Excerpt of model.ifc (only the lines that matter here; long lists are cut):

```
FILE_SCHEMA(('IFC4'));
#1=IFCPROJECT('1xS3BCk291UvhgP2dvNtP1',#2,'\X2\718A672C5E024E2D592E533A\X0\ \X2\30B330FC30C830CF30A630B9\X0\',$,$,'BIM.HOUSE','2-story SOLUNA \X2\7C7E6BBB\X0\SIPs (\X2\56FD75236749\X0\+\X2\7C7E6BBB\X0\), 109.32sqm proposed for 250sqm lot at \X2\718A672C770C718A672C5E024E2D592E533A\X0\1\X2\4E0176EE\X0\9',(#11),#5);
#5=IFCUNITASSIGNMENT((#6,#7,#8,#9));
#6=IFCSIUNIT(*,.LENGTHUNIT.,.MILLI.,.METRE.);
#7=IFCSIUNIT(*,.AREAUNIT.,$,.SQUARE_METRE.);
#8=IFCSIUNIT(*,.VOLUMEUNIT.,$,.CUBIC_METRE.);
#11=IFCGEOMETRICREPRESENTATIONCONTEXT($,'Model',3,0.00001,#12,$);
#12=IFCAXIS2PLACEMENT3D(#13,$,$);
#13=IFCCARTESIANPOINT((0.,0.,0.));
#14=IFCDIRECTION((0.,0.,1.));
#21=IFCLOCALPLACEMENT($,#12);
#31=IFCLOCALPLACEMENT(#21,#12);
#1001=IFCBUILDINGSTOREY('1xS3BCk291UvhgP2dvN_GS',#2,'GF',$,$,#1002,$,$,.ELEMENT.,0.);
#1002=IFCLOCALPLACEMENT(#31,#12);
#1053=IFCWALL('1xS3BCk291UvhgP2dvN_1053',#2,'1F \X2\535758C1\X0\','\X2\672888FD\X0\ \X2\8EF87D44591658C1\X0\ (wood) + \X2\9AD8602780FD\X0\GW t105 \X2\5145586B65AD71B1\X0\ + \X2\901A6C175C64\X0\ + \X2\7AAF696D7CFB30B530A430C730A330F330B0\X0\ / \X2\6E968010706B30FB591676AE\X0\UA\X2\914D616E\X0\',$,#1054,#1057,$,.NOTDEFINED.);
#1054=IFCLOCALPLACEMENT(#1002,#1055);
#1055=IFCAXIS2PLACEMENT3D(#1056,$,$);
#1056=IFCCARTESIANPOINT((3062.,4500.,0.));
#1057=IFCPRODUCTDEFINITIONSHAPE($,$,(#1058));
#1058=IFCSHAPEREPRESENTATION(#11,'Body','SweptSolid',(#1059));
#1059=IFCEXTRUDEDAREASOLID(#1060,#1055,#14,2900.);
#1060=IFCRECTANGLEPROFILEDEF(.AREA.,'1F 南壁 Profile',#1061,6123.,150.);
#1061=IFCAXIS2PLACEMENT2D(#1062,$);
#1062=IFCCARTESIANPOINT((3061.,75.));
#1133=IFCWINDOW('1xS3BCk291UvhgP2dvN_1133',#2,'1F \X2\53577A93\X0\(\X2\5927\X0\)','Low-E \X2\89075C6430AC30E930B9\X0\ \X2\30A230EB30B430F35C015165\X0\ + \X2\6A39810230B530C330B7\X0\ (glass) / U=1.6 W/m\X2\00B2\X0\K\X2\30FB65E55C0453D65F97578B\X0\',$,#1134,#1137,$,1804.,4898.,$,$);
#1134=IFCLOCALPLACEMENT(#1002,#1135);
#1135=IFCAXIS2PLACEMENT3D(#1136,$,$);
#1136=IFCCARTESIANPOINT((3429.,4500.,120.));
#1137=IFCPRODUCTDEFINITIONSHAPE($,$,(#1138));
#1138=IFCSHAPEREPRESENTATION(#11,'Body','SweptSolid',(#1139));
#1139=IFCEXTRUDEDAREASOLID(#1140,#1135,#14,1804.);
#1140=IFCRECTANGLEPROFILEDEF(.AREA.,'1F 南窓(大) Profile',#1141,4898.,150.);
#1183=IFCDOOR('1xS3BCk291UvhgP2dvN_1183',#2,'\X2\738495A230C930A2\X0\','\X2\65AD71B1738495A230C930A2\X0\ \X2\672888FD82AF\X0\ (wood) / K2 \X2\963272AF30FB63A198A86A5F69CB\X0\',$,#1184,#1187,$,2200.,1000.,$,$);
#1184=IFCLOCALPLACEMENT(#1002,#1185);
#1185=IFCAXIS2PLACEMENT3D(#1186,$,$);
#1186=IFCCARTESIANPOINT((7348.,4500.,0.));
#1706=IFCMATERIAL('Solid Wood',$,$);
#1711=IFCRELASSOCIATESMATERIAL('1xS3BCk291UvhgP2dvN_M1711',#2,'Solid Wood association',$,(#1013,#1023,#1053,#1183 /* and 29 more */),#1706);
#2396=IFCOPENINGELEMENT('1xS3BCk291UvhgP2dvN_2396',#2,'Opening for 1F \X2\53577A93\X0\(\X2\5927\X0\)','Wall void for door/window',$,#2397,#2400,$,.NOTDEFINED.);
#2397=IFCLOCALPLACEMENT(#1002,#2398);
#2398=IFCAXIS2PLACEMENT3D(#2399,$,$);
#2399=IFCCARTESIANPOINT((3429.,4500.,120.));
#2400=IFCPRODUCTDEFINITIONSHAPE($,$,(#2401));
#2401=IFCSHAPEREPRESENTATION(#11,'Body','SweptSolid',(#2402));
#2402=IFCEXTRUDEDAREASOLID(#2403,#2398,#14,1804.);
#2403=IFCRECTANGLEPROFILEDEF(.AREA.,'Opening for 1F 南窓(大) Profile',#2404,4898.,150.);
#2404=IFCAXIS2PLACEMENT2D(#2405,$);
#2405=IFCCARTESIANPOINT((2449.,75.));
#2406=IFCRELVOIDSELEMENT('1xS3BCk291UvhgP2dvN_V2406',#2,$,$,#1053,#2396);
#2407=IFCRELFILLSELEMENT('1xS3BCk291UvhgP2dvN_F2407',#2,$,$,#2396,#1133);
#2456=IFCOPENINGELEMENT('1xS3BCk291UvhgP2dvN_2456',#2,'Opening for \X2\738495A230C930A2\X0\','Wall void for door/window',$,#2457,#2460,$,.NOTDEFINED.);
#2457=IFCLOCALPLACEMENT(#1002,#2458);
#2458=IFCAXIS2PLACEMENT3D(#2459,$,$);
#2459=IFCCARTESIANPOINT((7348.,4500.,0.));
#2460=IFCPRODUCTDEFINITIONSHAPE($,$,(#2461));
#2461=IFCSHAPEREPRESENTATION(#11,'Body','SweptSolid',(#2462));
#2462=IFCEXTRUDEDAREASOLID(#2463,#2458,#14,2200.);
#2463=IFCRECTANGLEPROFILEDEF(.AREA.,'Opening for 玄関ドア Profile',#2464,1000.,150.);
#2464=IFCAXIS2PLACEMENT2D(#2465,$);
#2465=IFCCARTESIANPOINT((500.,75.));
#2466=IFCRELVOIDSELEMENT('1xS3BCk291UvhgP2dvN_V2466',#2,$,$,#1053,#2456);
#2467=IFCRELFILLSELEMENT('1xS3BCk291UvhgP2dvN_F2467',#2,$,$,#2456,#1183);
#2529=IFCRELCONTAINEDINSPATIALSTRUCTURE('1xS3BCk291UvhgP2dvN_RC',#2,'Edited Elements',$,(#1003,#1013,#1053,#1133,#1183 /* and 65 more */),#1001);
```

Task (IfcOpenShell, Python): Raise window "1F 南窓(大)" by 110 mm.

```python
import numpy as np
import ifcopenshell
import ifcopenshell.api.geometry
import ifcopenshell.util.placement
import ifcopenshell.util.unit

model = ifcopenshell.open("model.ifc")
unit_scale = ifcopenshell.util.unit.calculate_unit_scale(model)

window = model.by_id(1133)
opening = window.FillsVoids[0].RelatingOpeningElement
dz = 0.11 / unit_scale

shift = np.array([0.0, 0.0, dz])
# The window is not placed relative to its opening, so move both.
for product in (opening, window):
    matrix = ifcopenshell.util.placement.get_local_placement(product.ObjectPlacement)
    matrix[:3, 3] += shift
    ifcopenshell.api.geometry.edit_object_placement(model, product=product, matrix=matrix, is_si=False)

print(f"moved by {dz * unit_scale:+.3f} m")

model.write("model-out.ifc")
```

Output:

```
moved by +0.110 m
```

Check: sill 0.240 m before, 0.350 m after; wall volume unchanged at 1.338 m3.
